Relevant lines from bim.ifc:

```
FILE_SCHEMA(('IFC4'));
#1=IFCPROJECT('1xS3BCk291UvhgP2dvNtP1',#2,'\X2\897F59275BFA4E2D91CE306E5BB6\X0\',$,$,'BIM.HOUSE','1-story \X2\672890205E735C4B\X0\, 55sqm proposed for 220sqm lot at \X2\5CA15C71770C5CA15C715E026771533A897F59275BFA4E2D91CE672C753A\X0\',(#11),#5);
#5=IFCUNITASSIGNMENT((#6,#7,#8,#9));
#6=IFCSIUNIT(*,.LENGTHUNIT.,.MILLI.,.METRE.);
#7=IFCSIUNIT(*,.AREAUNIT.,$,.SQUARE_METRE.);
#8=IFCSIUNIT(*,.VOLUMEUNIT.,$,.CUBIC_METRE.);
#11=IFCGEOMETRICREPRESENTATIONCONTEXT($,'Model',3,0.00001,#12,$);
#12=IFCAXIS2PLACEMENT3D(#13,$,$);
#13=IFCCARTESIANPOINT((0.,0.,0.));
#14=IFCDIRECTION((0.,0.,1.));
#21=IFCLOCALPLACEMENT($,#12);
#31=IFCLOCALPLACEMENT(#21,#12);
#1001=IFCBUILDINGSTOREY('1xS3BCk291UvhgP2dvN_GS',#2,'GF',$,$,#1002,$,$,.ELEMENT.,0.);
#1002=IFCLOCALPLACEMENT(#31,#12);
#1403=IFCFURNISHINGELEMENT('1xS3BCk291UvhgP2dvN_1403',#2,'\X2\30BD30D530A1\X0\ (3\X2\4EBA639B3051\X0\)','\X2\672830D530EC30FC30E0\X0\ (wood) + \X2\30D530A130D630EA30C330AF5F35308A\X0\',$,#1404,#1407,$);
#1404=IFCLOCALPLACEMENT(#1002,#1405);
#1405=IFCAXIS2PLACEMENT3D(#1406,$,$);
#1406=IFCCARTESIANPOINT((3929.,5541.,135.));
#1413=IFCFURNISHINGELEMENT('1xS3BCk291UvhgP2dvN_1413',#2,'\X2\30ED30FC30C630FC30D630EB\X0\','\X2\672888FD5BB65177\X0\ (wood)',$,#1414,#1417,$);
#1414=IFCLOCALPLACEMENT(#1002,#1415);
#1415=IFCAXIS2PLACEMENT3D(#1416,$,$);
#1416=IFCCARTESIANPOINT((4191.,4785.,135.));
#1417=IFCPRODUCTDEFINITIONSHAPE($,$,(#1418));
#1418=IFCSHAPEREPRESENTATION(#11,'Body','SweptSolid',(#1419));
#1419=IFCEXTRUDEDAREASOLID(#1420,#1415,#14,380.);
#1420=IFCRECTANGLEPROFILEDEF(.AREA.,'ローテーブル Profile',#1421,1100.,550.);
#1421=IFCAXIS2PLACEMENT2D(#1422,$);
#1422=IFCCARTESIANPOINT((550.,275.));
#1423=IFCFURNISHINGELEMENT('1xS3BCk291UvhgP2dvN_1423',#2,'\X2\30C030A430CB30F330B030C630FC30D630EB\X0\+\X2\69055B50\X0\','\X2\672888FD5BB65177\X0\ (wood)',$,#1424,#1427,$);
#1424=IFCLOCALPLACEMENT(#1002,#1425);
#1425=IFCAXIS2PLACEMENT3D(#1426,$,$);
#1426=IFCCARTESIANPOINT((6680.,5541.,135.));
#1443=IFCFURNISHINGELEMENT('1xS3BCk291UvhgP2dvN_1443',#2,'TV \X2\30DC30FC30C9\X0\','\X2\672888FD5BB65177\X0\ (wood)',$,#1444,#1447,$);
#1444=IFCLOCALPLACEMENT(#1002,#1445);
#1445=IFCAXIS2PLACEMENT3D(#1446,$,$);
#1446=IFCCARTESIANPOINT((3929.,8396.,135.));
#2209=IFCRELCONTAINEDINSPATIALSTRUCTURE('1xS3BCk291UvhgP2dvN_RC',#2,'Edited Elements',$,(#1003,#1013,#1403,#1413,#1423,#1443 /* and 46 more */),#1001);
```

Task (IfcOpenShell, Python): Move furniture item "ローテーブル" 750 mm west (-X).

```python
import ifcopenshell
import ifcopenshell.api.geometry
import ifcopenshell.util.placement
import ifcopenshell.util.unit

model = ifcopenshell.open("bim.ifc")
unit_scale = ifcopenshell.util.unit.calculate_unit_scale(model)

item = model.by_guid("1xS3BCk291UvhgP2dvN_1413")
matrix = ifcopenshell.util.placement.get_local_placement(item.ObjectPlacement)
matrix[0, 3] -= 0.75 / unit_scale
ifcopenshell.api.geometry.edit_object_placement(model, product=item, matrix=matrix, is_si=False)

print(ifcopenshell.util.placement.get_local_placement(item.ObjectPlacement).round(3) + 0.0)

model.write("bim_rev.ifc")
```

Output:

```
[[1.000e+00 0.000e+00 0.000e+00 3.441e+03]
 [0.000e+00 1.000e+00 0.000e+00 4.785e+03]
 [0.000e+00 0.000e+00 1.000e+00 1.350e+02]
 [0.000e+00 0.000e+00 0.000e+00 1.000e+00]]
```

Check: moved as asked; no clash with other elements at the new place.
